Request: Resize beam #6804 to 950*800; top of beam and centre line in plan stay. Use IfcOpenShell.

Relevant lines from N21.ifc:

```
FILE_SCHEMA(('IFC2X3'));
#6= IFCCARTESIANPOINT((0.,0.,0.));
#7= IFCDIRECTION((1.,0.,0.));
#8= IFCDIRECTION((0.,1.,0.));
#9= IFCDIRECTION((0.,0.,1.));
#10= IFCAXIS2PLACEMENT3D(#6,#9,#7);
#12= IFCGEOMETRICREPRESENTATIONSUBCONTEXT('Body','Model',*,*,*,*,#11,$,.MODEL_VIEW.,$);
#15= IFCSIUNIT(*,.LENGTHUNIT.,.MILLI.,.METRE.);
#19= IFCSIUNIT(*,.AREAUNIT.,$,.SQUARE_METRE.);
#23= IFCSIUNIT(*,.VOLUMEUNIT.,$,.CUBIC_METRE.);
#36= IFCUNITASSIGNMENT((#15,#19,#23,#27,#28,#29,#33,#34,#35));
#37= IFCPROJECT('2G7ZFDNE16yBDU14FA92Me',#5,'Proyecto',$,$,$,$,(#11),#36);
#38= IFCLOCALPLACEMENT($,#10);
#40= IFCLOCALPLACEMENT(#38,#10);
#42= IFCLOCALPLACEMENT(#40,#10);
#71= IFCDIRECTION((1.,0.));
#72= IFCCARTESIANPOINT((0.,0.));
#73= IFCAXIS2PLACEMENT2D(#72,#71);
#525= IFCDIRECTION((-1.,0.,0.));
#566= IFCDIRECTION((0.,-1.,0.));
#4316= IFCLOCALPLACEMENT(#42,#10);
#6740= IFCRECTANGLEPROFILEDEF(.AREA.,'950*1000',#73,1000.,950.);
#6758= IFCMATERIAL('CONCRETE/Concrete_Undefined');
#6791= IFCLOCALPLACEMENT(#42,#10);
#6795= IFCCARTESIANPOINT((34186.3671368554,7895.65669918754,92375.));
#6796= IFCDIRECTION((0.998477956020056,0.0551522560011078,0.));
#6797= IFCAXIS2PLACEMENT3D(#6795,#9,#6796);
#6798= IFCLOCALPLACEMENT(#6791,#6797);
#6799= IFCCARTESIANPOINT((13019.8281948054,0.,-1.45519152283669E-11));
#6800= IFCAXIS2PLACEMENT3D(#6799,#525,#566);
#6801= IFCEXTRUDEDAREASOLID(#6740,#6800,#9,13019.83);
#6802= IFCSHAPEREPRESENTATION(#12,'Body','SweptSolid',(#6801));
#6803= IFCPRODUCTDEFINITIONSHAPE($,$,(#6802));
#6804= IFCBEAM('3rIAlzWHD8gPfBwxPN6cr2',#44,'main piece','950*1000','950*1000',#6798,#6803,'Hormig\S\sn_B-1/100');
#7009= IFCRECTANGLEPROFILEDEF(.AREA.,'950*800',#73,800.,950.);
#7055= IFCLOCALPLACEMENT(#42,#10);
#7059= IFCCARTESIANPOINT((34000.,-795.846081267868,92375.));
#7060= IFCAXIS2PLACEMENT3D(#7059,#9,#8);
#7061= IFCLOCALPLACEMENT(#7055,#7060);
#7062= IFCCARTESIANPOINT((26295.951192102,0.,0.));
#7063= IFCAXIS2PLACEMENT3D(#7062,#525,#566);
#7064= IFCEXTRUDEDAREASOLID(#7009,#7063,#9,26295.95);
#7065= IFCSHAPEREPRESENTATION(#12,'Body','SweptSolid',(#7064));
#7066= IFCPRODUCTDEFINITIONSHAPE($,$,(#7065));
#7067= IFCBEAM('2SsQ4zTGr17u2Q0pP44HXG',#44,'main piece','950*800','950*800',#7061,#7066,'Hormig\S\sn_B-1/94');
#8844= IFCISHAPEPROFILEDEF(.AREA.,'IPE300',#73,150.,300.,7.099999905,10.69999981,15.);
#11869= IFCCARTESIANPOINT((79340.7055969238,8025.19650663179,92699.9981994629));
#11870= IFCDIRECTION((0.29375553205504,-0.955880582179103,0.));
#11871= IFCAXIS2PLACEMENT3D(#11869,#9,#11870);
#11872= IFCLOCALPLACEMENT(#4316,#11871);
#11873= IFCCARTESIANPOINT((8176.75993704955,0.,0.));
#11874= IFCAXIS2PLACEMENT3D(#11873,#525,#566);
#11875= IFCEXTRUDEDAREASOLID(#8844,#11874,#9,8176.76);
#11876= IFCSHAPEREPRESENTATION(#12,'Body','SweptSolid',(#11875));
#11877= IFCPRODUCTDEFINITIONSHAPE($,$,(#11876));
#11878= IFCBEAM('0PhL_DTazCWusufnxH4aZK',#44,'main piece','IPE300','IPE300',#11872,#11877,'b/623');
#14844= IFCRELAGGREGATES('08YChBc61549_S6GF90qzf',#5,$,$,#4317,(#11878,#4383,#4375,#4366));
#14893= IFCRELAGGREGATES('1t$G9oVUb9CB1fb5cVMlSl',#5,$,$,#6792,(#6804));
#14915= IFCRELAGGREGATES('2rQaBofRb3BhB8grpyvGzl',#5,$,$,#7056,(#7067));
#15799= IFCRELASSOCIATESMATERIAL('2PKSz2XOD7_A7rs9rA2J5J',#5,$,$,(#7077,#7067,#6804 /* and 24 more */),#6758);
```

```python
import ifcopenshell
import ifcopenshell.util.element
import ifcopenshell.util.representation

model = ifcopenshell.open("N21.ifc")

member = model.by_guid("3rIAlzWHD8gPfBwxPN6cr2")
source = next(p for p in model.by_type("IfcRectangleProfileDef") if p.ProfileName == "950*800")

body = ifcopenshell.util.representation.get_representation(member, "Model", "Body")
solid = body.Items[0]
old_profile = solid.SweptArea

# Copy the section's sizes but keep this member's own profile position.
profile = ifcopenshell.util.element.copy(model, source)
# Profiles are centred, so shift by half the change in depth to hold the top.
shift = (old_profile.YDim - profile.YDim) / 2
x, y = old_profile.Position.Location.Coordinates
up = (0.0, 1.0)  # upwards, in the solid's own plane
location = model.createIfcCartesianPoint((x + up[0] * shift, y + up[1] * shift))
profile.Position = model.createIfcAxis2Placement2D(location, old_profile.Position.RefDirection)
solid.SweptArea = profile
if not model.get_total_inverses(old_profile):
    ifcopenshell.util.element.remove_deep2(model, old_profile)
member.Description = member.Description.replace("950*1000", "950*800")
member.ObjectType = member.ObjectType.replace("950*1000", "950*800")

print(solid.SweptArea)

model.write("N21-out.ifc")
```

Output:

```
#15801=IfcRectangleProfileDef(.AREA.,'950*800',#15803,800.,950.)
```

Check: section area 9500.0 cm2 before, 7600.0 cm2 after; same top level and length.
